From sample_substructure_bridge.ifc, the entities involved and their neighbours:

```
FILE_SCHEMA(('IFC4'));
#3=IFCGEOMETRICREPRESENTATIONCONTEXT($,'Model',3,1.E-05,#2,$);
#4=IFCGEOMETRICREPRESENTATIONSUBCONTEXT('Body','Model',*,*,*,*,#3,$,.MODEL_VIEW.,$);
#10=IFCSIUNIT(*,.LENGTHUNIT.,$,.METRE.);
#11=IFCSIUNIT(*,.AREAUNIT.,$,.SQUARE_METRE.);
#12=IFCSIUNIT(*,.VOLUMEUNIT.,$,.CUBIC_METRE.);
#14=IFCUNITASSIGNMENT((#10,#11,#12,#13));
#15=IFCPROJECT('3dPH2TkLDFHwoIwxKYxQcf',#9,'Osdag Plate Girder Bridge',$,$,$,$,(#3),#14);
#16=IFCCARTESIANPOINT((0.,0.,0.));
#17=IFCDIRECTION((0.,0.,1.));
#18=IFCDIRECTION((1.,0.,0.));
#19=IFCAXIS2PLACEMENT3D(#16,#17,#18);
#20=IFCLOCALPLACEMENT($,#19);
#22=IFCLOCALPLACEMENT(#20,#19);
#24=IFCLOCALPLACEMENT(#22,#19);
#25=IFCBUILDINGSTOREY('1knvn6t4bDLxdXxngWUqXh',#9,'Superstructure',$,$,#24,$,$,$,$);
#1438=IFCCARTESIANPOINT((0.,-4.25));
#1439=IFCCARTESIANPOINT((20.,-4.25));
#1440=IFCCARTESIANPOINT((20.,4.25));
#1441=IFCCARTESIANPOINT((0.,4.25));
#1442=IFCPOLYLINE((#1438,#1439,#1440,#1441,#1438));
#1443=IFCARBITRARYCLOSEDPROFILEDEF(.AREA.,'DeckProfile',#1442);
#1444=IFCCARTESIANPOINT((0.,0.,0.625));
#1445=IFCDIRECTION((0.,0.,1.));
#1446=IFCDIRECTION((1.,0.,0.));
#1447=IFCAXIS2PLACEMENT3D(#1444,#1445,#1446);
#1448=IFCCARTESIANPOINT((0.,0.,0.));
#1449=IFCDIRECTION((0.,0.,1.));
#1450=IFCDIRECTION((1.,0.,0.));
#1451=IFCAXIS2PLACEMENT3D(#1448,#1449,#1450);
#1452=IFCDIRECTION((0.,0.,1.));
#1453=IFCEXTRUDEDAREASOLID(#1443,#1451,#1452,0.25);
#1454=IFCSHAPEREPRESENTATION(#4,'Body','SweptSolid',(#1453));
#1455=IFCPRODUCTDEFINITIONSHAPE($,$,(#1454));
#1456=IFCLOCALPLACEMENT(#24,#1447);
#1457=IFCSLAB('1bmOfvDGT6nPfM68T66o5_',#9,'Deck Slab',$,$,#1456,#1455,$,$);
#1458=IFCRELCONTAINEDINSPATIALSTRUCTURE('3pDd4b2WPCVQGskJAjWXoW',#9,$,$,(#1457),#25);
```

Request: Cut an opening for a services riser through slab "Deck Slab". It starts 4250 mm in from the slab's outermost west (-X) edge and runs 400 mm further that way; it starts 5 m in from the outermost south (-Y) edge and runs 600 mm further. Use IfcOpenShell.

```python
import numpy as np
import ifcopenshell
import ifcopenshell.api.feature
import ifcopenshell.api.geometry
import ifcopenshell.api.root
import ifcopenshell.geom
import ifcopenshell.util.placement
import ifcopenshell.util.representation
import ifcopenshell.util.shape
import ifcopenshell.util.unit

model = ifcopenshell.open("sample_substructure_bridge.ifc")
unit_scale = ifcopenshell.util.unit.calculate_unit_scale(model)
settings = ifcopenshell.geom.settings()


def volume(element):
    """Net volume in cubic metres, openings subtracted."""
    shape = ifcopenshell.geom.create_shape(settings, element)
    return ifcopenshell.util.shape.get_volume(shape.geometry)


slab = model.by_id(1457)
before = volume(slab)

# Extent in the slab's own axes, in metres. The edges named are its -X and -Y sides.
slab_shape = ifcopenshell.geom.create_shape(settings, slab)
vertices = ifcopenshell.util.shape.get_vertices(slab_shape.geometry)
x_min, y_min, bottom = vertices.min(axis=0)
top = vertices[:, 2].max()

opening = ifcopenshell.api.root.create_entity(model, ifc_class="IfcOpeningElement", name="Services riser opening", predefined_type="OPENING")
context = ifcopenshell.util.representation.get_context(model, "Model", "Body", "MODEL_VIEW")
width, depth = 0.4, 0.6
outline = [(0.0, 0.0), (width, 0.0), (width, depth), (0.0, depth), (0.0, 0.0)]
# Overshoot both faces by 50 mm so the cut is clean.
shape = ifcopenshell.api.geometry.add_slab_representation(
    model, context=context, depth=top - bottom + 0.1, polyline=outline
)
ifcopenshell.api.geometry.assign_representation(model, product=opening, representation=shape)

matrix = ifcopenshell.util.placement.get_local_placement(slab.ObjectPlacement)
matrix[:, 3] = matrix @ np.append(np.array([x_min + 4.25, y_min + 5, bottom - 0.05]) / unit_scale, 1.0)
ifcopenshell.api.geometry.edit_object_placement(model, product=opening, matrix=matrix, is_si=False)
ifcopenshell.api.feature.add_feature(model, feature=opening, element=slab)

after = volume(slab)

print(f"slab volume {before:.3f} -> {after:.3f} m3")

model.write("sample_substructure_bridge_edited.ifc")
```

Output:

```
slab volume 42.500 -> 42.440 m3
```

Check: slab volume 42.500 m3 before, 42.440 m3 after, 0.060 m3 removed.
